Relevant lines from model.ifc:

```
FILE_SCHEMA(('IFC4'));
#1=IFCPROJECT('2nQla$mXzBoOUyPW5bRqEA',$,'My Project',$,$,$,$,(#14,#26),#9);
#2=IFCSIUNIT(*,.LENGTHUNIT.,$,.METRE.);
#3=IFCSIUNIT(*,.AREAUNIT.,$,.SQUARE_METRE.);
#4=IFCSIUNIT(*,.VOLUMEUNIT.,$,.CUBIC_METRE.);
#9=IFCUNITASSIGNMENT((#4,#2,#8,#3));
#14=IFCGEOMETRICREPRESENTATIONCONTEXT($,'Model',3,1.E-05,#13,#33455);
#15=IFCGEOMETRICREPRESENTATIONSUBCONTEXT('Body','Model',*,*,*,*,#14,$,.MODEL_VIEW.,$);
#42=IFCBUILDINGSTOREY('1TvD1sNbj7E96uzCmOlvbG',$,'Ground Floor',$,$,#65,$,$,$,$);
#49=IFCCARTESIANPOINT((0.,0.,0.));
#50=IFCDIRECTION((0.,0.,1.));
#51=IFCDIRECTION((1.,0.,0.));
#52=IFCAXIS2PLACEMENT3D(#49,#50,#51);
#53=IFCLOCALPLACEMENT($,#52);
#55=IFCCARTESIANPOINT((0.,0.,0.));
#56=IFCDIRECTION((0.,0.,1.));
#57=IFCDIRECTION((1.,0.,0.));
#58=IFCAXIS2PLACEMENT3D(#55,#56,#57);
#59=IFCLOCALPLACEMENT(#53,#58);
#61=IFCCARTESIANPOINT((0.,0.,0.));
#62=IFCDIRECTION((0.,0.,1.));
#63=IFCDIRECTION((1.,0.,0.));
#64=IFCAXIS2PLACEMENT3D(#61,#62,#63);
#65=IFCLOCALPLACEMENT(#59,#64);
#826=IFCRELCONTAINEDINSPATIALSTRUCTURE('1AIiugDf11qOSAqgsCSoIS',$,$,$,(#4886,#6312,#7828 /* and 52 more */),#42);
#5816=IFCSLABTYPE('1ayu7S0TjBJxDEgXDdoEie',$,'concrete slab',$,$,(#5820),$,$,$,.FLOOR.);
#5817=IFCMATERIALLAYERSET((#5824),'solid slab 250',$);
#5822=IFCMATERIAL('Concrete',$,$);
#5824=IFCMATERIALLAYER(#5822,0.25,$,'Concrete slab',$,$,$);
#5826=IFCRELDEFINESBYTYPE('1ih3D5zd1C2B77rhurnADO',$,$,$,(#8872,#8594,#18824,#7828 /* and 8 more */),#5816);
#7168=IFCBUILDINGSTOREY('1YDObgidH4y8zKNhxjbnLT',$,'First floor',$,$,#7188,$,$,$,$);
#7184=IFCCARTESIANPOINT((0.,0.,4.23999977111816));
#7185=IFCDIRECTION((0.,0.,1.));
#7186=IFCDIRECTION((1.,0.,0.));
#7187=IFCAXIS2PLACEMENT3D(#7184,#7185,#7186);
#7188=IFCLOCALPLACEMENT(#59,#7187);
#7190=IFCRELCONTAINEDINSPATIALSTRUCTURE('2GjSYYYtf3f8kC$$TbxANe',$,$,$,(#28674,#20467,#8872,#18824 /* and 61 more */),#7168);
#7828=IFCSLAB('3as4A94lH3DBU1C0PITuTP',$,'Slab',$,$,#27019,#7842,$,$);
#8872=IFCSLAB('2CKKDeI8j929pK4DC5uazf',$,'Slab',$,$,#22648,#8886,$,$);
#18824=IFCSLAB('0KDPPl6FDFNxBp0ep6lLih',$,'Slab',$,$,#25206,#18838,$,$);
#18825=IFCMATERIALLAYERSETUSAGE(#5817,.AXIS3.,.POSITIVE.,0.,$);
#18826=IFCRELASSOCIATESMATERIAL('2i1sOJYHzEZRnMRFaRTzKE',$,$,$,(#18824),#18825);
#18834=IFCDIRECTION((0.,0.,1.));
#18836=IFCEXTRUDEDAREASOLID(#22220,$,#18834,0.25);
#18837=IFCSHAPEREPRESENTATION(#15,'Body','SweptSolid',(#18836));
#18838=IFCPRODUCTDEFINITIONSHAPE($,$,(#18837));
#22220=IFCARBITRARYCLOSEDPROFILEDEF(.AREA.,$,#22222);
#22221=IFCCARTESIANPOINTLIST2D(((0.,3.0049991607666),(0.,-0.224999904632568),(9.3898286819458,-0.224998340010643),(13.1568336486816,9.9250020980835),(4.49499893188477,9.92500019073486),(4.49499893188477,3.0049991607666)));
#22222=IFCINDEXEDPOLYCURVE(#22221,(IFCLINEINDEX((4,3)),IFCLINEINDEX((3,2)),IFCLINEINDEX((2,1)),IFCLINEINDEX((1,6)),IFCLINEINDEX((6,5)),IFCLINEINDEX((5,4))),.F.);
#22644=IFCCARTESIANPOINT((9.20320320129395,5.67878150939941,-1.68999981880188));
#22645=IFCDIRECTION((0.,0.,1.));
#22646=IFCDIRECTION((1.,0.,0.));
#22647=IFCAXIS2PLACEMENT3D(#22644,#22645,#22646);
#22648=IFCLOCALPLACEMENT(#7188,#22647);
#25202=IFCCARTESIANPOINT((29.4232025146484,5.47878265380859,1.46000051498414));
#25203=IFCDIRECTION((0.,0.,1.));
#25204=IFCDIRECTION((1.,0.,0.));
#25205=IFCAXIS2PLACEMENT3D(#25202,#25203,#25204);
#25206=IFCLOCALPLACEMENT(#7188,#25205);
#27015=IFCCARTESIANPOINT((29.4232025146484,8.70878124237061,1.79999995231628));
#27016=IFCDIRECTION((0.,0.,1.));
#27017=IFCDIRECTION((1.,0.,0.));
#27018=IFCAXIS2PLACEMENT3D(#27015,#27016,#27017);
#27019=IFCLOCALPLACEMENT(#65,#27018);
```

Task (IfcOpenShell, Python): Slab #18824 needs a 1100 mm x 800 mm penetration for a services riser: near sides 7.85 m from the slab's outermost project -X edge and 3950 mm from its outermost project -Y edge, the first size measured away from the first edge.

```python
import numpy as np
import ifcopenshell
import ifcopenshell.api.feature
import ifcopenshell.api.geometry
import ifcopenshell.api.root
import ifcopenshell.geom
import ifcopenshell.util.placement
import ifcopenshell.util.representation
import ifcopenshell.util.shape
import ifcopenshell.util.unit

model = ifcopenshell.open("model.ifc")
unit_scale = ifcopenshell.util.unit.calculate_unit_scale(model)
settings = ifcopenshell.geom.settings()


def volume(element):
    """Net volume in cubic metres, openings subtracted."""
    shape = ifcopenshell.geom.create_shape(settings, element)
    return ifcopenshell.util.shape.get_volume(shape.geometry)


slab = model.by_guid("0KDPPl6FDFNxBp0ep6lLih")
before = volume(slab)

# Extent in the slab's own axes, in metres. The edges named are its -X and -Y sides.
slab_shape = ifcopenshell.geom.create_shape(settings, slab)
vertices = ifcopenshell.util.shape.get_vertices(slab_shape.geometry)
x_min, y_min, bottom = vertices.min(axis=0)
top = vertices[:, 2].max()

opening = ifcopenshell.api.root.create_entity(model, ifc_class="IfcOpeningElement", name="Services riser opening", predefined_type="OPENING")
context = ifcopenshell.util.representation.get_context(model, "Model", "Body", "MODEL_VIEW")
width, depth = 1.1, 0.8
outline = [(0.0, 0.0), (width, 0.0), (width, depth), (0.0, depth), (0.0, 0.0)]
# Overshoot both faces by 50 mm so the cut is clean.
shape = ifcopenshell.api.geometry.add_slab_representation(
    model, context=context, depth=top - bottom + 0.1, polyline=outline
)
ifcopenshell.api.geometry.assign_representation(model, product=opening, representation=shape)

matrix = ifcopenshell.util.placement.get_local_placement(slab.ObjectPlacement)
matrix[:, 3] = matrix @ np.append(np.array([x_min + 7.85, y_min + 3.95, bottom - 0.05]) / unit_scale, 1.0)
ifcopenshell.api.geometry.edit_object_placement(model, product=opening, matrix=matrix, is_si=False)
ifcopenshell.api.feature.add_feature(model, feature=opening, element=slab)

after = volume(slab)

print(f"slab volume {before:.3f} -> {after:.3f} m3")

model.write("model_rev.ifc")
```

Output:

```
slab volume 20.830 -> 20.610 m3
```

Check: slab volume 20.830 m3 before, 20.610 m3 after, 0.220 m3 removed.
